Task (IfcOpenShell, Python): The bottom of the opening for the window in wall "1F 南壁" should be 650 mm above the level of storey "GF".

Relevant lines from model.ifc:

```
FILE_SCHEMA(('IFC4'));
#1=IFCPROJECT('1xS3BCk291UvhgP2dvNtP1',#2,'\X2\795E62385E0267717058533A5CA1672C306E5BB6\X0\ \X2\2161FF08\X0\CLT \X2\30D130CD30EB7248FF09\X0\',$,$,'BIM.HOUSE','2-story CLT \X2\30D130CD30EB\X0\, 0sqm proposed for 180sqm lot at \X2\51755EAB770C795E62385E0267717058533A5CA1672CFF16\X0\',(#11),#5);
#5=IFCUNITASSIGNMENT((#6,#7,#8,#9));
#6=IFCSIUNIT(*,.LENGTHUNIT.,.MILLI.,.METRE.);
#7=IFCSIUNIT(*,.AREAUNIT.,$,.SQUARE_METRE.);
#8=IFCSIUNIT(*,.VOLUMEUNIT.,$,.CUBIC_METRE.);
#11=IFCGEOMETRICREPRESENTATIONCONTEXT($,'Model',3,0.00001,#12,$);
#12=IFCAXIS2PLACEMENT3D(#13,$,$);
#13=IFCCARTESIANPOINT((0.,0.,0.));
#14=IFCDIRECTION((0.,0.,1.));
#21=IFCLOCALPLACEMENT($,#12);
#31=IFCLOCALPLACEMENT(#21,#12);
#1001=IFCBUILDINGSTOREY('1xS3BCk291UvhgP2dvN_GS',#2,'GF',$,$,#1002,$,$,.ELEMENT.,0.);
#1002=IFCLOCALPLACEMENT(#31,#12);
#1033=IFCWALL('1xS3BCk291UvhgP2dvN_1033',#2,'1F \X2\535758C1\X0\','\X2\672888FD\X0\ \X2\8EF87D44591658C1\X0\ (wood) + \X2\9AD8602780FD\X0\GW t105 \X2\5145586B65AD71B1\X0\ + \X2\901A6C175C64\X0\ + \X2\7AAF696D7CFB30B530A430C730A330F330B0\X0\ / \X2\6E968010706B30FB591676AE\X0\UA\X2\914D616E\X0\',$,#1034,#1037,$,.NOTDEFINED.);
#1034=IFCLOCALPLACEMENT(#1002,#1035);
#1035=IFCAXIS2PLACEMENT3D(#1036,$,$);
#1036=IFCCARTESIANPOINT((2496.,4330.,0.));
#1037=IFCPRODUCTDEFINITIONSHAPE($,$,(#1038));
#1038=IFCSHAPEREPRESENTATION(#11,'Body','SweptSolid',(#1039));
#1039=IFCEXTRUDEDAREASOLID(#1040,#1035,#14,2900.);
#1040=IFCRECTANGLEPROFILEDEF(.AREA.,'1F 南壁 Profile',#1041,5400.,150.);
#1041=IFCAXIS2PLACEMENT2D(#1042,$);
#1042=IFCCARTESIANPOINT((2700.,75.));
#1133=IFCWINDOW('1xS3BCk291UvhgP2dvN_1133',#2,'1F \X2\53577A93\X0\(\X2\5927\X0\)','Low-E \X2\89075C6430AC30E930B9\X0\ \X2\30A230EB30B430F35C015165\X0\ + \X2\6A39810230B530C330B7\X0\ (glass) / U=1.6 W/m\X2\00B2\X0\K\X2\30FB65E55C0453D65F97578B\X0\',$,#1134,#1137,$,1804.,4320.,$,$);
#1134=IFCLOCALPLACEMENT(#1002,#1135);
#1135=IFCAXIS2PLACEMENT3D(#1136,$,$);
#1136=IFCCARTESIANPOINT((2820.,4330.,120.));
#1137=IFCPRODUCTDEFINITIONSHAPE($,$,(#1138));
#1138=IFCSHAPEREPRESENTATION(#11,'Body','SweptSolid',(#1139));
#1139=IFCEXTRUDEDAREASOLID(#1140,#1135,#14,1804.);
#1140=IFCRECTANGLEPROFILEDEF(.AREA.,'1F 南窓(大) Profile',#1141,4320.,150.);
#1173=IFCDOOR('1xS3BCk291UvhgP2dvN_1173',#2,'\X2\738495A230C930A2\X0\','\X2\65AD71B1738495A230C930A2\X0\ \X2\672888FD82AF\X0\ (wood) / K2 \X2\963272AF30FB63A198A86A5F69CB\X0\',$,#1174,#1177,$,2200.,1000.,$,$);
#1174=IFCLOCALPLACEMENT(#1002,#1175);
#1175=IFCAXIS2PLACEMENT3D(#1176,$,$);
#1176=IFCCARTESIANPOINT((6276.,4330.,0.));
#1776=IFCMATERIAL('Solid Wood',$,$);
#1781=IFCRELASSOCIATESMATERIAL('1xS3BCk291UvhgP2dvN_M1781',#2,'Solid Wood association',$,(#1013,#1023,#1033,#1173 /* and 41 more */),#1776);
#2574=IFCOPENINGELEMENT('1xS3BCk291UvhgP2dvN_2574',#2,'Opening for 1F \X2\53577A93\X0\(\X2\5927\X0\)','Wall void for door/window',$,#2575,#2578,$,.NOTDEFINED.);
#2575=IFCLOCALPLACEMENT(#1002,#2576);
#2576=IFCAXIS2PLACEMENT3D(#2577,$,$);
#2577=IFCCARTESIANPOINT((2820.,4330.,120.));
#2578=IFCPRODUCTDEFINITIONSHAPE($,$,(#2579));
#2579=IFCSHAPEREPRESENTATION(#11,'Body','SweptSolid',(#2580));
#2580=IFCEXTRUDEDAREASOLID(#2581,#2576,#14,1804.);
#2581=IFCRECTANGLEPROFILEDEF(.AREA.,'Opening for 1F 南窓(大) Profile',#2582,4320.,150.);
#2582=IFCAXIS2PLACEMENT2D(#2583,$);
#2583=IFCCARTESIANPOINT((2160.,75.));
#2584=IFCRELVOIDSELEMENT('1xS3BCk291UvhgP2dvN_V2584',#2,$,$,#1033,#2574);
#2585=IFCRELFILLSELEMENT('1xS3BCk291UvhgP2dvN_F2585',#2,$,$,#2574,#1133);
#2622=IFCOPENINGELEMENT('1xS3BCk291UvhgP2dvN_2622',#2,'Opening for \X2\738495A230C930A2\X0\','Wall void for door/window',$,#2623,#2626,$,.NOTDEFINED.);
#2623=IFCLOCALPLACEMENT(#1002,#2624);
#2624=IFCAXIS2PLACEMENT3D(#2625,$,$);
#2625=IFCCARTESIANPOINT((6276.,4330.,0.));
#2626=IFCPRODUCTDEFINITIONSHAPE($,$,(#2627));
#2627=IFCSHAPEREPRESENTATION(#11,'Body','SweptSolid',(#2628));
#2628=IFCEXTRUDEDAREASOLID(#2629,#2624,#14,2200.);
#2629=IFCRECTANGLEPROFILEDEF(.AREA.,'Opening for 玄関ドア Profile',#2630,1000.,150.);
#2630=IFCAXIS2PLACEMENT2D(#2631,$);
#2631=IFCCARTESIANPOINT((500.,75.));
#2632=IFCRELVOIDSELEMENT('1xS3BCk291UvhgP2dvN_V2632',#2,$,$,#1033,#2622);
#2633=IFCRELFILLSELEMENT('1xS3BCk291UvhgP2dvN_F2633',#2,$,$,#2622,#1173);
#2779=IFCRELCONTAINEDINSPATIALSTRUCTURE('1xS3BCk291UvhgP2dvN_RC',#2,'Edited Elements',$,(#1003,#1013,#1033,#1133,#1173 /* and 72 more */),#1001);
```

```python
import numpy as np
import ifcopenshell
import ifcopenshell.api.geometry
import ifcopenshell.geom
import ifcopenshell.util.element
import ifcopenshell.util.placement
import ifcopenshell.util.shape
import ifcopenshell.util.unit

model = ifcopenshell.open("model.ifc")
unit_scale = ifcopenshell.util.unit.calculate_unit_scale(model)

window = model.by_guid("1xS3BCk291UvhgP2dvN_1133")
opening = window.FillsVoids[0].RelatingOpeningElement
storey = ifcopenshell.util.element.get_container(window, ifc_class="IfcBuildingStorey")
level = ifcopenshell.util.placement.get_local_placement(storey.ObjectPlacement)[2, 3]

# The opening's origin need not be at the sill, so measure its lowest point.
shape = ifcopenshell.geom.create_shape(ifcopenshell.geom.settings(), opening)
bottom = ifcopenshell.util.shape.get_shape_bottom_elevation(shape, shape.geometry) / unit_scale
dz = level + 650.0 - bottom

shift = np.array([0.0, 0.0, dz])
# The window is not placed relative to its opening, so move both.
for product in (opening, window):
    matrix = ifcopenshell.util.placement.get_local_placement(product.ObjectPlacement)
    matrix[:3, 3] += shift
    ifcopenshell.api.geometry.edit_object_placement(model, product=product, matrix=matrix, is_si=False)

print(f"moved by {dz * unit_scale:+.3f} m")

model.write("model_updated.ifc")
```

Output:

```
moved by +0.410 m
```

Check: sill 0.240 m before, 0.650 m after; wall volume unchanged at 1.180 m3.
